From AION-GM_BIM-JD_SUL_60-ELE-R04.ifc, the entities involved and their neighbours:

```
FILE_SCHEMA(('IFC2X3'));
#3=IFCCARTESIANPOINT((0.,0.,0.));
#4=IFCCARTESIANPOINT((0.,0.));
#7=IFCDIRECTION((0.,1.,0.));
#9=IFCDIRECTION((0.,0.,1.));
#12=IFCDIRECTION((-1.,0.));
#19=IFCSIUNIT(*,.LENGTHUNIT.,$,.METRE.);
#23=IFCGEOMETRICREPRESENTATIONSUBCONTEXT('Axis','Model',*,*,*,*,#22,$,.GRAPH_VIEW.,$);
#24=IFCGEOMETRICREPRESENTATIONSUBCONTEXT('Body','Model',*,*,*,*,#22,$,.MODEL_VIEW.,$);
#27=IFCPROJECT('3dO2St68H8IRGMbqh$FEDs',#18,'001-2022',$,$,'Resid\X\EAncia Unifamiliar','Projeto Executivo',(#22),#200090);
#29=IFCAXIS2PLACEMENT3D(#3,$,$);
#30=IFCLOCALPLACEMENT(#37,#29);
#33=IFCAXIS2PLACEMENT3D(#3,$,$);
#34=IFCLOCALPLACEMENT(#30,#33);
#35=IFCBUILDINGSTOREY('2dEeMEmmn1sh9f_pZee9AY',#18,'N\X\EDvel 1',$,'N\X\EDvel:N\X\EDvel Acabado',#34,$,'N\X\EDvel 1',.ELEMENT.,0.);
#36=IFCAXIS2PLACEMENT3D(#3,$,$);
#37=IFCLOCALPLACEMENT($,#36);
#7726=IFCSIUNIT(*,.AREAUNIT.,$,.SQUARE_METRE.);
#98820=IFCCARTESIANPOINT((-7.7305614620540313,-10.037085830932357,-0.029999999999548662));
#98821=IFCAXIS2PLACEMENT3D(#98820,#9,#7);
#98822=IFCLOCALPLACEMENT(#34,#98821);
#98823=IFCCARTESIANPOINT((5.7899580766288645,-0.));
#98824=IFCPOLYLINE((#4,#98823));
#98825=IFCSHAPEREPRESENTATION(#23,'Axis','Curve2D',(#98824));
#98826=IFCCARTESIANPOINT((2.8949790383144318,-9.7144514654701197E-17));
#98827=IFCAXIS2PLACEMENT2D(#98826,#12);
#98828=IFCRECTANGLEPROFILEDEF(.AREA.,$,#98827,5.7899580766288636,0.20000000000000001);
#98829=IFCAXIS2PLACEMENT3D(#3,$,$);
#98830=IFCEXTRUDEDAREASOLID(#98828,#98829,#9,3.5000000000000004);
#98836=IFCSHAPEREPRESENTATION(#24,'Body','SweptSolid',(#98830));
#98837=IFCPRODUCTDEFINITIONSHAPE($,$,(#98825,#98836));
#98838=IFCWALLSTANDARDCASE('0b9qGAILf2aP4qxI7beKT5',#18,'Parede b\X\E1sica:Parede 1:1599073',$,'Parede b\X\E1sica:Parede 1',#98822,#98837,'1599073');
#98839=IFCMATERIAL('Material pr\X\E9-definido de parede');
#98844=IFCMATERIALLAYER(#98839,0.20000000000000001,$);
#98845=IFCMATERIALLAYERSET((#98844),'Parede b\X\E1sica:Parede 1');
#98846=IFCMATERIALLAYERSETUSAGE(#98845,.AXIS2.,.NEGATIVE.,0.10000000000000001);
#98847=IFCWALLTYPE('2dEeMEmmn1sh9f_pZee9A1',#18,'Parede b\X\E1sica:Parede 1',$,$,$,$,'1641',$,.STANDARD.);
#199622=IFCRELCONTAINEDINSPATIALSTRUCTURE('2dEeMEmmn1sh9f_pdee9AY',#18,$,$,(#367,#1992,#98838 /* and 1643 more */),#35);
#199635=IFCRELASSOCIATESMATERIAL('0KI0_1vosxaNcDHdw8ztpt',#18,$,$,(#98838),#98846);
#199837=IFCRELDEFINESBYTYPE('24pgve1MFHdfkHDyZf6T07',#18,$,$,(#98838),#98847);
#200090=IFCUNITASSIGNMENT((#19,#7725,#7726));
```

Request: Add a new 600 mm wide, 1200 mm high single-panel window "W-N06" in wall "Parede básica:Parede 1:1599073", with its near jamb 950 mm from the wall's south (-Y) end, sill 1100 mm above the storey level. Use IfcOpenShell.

```python
import numpy as np
import ifcopenshell
import ifcopenshell.api.feature
import ifcopenshell.api.geometry
import ifcopenshell.api.root
import ifcopenshell.api.spatial
import ifcopenshell.api.type
import ifcopenshell.geom
import ifcopenshell.util.element
import ifcopenshell.util.placement
import ifcopenshell.util.representation
import ifcopenshell.util.shape
import ifcopenshell.util.unit

model = ifcopenshell.open("AION-GM_BIM-JD_SUL_60-ELE-R04.ifc")
unit_scale = ifcopenshell.util.unit.calculate_unit_scale(model)
settings = ifcopenshell.geom.settings()


def volume(element):
    """Net volume in cubic metres, openings subtracted."""
    shape = ifcopenshell.geom.create_shape(settings, element)
    return ifcopenshell.util.shape.get_volume(shape.geometry)


wall = model.by_guid("0b9qGAILf2aP4qxI7beKT5")
storey = ifcopenshell.util.element.get_container(wall, ifc_class="IfcBuildingStorey")
context = ifcopenshell.util.representation.get_context(model, "Model", "Body", "MODEL_VIEW")
before = volume(wall)

width, height, from_end, sill = 0.6, 1.2, 0.95, 1.1  # metres

# The wall runs along its own X axis, and the end named is its -X end.
wall_shape = ifcopenshell.geom.create_shape(settings, wall)
x, y, z = ifcopenshell.util.shape.get_vertices(wall_shape.geometry).T
start = x.min() + from_end
face, thickness = float(y.min()), float(y.max() - y.min())
wall_matrix = ifcopenshell.util.placement.get_local_placement(wall.ObjectPlacement)
level = ifcopenshell.util.placement.get_local_placement(storey.ObjectPlacement)[2, 3]


def in_wall(x, y):
    """Placement at x, y metres in the wall's axes, at sill height."""
    matrix = wall_matrix.copy()
    matrix[:, 3] = wall_matrix @ np.array([x / unit_scale, y / unit_scale, 0.0, 1.0])
    matrix[2, 3] = level + sill / unit_scale
    return matrix


# Opening: a box that overshoots both wall faces by 50 mm.
opening = ifcopenshell.api.root.create_entity(model, ifc_class="IfcOpeningElement")
box = ifcopenshell.api.geometry.add_wall_representation(
    model, context=context, length=width, height=height, thickness=thickness + 0.1
)
ifcopenshell.api.geometry.assign_representation(model, product=opening, representation=box)
ifcopenshell.api.geometry.edit_object_placement(model, product=opening, matrix=in_wall(start, face - 0.05), is_si=False)
ifcopenshell.api.feature.add_feature(model, feature=opening, element=wall)

window = ifcopenshell.api.root.create_entity(model, ifc_class="IfcWindow", name="W-N06")
window.OverallWidth, window.OverallHeight = width / unit_scale, height / unit_scale
body = ifcopenshell.api.geometry.add_window_representation(
    model,
    context=context,
    overall_width=window.OverallWidth,
    overall_height=window.OverallHeight,
    partition_type="SINGLE_PANEL",
)
ifcopenshell.api.geometry.assign_representation(model, product=window, representation=body)
ifcopenshell.api.spatial.assign_container(model, products=[window], relating_structure=storey)
fills = ifcopenshell.api.feature.add_filling(model, opening=opening, element=window)
fills.OwnerHistory = window.OwnerHistory  # required in IFC2X3

# IFC2X3 keeps the operation on the window style.
style = ifcopenshell.api.root.create_entity(model, ifc_class="IfcWindowStyle", name="W-N06")
style.OperationType, style.ConstructionType = "SINGLE_PANEL", "NOTDEFINED"
style.ParameterTakesPrecedence = style.Sizeable = False
ifcopenshell.api.type.assign_type(model, related_objects=[window], relating_type=style)

# Centre the window in the wall's thickness.
ifcopenshell.api.geometry.edit_object_placement(model, product=window, matrix=in_wall(start, face), is_si=False)
window_shape = ifcopenshell.geom.create_shape(settings, window)
depth = ifcopenshell.util.shape.get_vertices(window_shape.geometry)[:, 1]
offset = face + thickness / 2 - (depth.min() + depth.max()) / 2
ifcopenshell.api.geometry.edit_object_placement(model, product=window, matrix=in_wall(start, offset), is_si=False)

after = volume(wall)

print(f"wall volume {before:.3f} -> {after:.3f} m3")

model.write("AION-GM_BIM-JD_SUL_60-ELE-R04_rev.ifc")
```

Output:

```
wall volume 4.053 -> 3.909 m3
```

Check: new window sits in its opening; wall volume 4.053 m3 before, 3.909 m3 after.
